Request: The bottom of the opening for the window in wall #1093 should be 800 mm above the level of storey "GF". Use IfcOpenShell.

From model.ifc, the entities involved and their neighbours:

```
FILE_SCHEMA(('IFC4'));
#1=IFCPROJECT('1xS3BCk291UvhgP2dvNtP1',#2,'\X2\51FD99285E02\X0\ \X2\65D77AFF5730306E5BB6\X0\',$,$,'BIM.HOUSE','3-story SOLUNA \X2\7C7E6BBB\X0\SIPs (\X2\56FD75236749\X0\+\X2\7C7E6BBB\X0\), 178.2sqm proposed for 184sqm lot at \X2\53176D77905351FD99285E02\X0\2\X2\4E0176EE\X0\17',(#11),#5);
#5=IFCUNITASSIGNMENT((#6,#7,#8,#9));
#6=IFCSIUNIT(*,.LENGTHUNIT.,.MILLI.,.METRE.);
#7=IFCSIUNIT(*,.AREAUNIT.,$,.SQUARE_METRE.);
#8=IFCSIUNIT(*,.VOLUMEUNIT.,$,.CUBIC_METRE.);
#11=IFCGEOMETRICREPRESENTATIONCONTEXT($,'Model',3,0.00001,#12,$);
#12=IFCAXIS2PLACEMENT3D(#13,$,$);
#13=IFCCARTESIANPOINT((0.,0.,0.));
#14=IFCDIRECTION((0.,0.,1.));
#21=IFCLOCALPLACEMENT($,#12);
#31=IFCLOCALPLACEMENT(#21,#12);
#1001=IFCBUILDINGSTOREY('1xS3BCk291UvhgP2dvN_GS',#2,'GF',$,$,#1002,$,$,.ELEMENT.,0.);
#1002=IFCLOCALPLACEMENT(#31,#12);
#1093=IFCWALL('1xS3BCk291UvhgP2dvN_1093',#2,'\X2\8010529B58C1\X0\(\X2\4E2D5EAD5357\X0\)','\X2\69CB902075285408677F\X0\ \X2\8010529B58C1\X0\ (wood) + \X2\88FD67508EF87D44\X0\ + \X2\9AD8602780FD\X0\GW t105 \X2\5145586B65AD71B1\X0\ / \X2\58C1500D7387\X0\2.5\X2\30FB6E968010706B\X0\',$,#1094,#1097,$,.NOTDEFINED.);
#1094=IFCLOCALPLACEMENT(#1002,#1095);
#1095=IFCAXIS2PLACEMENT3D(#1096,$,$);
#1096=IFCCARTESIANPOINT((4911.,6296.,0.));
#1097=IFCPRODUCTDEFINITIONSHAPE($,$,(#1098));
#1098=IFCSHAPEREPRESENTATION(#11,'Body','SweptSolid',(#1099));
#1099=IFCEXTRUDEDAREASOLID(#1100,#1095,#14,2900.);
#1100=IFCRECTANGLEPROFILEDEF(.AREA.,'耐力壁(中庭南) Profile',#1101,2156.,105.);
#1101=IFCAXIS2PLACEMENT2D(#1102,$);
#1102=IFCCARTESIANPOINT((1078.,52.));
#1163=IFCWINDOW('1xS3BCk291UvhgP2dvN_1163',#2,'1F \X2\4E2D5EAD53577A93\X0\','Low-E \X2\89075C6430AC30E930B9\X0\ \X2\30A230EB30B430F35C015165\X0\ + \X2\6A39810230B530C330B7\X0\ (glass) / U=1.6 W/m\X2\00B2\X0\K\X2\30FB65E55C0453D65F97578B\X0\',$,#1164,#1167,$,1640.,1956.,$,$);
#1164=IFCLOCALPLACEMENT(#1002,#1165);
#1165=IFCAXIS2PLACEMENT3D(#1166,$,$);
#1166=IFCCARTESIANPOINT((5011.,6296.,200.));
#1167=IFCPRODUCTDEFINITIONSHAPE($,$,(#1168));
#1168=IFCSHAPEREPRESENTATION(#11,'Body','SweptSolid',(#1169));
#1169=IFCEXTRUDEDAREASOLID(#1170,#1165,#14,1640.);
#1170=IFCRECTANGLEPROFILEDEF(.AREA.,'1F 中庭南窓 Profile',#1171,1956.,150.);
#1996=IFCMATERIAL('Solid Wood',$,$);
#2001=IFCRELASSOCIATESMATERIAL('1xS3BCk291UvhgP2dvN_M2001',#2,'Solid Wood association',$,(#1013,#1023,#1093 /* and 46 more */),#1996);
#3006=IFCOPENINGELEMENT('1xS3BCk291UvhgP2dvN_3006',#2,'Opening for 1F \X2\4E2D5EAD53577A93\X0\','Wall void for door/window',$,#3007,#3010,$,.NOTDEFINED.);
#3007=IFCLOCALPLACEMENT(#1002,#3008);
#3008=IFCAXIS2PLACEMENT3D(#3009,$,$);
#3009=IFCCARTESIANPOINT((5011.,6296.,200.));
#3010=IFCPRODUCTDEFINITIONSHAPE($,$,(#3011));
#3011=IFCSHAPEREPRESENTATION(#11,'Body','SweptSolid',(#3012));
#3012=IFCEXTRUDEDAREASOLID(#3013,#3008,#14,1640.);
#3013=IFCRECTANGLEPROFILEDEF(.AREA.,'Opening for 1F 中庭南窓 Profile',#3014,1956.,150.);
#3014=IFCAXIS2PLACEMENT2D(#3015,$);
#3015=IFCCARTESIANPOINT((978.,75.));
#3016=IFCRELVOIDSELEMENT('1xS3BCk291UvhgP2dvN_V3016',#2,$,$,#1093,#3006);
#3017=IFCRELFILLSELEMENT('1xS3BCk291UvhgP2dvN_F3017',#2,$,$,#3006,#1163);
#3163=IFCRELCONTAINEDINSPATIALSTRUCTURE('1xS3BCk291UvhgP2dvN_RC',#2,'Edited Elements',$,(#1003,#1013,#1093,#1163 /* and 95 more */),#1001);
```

```python
import numpy as np
import ifcopenshell
import ifcopenshell.api.geometry
import ifcopenshell.geom
import ifcopenshell.util.element
import ifcopenshell.util.placement
import ifcopenshell.util.shape
import ifcopenshell.util.unit

model = ifcopenshell.open("model.ifc")
unit_scale = ifcopenshell.util.unit.calculate_unit_scale(model)

window = model.by_guid("1xS3BCk291UvhgP2dvN_1163")
opening = window.FillsVoids[0].RelatingOpeningElement
storey = ifcopenshell.util.element.get_container(window, ifc_class="IfcBuildingStorey")
level = ifcopenshell.util.placement.get_local_placement(storey.ObjectPlacement)[2, 3]

# The opening's origin need not be at the sill, so measure its lowest point.
shape = ifcopenshell.geom.create_shape(ifcopenshell.geom.settings(), opening)
bottom = ifcopenshell.util.shape.get_shape_bottom_elevation(shape, shape.geometry) / unit_scale
dz = level + 0.8 / unit_scale - bottom

shift = np.array([0.0, 0.0, dz])
# The window is not placed relative to its opening, so move both.
for product in (opening, window):
    matrix = ifcopenshell.util.placement.get_local_placement(product.ObjectPlacement)
    matrix[:3, 3] += shift
    ifcopenshell.api.geometry.edit_object_placement(model, product=product, matrix=matrix, is_si=False)

print(f"moved by {dz * unit_scale:+.3f} m")

model.write("model_updated.ifc")
```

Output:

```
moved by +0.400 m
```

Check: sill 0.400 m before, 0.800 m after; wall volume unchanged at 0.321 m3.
